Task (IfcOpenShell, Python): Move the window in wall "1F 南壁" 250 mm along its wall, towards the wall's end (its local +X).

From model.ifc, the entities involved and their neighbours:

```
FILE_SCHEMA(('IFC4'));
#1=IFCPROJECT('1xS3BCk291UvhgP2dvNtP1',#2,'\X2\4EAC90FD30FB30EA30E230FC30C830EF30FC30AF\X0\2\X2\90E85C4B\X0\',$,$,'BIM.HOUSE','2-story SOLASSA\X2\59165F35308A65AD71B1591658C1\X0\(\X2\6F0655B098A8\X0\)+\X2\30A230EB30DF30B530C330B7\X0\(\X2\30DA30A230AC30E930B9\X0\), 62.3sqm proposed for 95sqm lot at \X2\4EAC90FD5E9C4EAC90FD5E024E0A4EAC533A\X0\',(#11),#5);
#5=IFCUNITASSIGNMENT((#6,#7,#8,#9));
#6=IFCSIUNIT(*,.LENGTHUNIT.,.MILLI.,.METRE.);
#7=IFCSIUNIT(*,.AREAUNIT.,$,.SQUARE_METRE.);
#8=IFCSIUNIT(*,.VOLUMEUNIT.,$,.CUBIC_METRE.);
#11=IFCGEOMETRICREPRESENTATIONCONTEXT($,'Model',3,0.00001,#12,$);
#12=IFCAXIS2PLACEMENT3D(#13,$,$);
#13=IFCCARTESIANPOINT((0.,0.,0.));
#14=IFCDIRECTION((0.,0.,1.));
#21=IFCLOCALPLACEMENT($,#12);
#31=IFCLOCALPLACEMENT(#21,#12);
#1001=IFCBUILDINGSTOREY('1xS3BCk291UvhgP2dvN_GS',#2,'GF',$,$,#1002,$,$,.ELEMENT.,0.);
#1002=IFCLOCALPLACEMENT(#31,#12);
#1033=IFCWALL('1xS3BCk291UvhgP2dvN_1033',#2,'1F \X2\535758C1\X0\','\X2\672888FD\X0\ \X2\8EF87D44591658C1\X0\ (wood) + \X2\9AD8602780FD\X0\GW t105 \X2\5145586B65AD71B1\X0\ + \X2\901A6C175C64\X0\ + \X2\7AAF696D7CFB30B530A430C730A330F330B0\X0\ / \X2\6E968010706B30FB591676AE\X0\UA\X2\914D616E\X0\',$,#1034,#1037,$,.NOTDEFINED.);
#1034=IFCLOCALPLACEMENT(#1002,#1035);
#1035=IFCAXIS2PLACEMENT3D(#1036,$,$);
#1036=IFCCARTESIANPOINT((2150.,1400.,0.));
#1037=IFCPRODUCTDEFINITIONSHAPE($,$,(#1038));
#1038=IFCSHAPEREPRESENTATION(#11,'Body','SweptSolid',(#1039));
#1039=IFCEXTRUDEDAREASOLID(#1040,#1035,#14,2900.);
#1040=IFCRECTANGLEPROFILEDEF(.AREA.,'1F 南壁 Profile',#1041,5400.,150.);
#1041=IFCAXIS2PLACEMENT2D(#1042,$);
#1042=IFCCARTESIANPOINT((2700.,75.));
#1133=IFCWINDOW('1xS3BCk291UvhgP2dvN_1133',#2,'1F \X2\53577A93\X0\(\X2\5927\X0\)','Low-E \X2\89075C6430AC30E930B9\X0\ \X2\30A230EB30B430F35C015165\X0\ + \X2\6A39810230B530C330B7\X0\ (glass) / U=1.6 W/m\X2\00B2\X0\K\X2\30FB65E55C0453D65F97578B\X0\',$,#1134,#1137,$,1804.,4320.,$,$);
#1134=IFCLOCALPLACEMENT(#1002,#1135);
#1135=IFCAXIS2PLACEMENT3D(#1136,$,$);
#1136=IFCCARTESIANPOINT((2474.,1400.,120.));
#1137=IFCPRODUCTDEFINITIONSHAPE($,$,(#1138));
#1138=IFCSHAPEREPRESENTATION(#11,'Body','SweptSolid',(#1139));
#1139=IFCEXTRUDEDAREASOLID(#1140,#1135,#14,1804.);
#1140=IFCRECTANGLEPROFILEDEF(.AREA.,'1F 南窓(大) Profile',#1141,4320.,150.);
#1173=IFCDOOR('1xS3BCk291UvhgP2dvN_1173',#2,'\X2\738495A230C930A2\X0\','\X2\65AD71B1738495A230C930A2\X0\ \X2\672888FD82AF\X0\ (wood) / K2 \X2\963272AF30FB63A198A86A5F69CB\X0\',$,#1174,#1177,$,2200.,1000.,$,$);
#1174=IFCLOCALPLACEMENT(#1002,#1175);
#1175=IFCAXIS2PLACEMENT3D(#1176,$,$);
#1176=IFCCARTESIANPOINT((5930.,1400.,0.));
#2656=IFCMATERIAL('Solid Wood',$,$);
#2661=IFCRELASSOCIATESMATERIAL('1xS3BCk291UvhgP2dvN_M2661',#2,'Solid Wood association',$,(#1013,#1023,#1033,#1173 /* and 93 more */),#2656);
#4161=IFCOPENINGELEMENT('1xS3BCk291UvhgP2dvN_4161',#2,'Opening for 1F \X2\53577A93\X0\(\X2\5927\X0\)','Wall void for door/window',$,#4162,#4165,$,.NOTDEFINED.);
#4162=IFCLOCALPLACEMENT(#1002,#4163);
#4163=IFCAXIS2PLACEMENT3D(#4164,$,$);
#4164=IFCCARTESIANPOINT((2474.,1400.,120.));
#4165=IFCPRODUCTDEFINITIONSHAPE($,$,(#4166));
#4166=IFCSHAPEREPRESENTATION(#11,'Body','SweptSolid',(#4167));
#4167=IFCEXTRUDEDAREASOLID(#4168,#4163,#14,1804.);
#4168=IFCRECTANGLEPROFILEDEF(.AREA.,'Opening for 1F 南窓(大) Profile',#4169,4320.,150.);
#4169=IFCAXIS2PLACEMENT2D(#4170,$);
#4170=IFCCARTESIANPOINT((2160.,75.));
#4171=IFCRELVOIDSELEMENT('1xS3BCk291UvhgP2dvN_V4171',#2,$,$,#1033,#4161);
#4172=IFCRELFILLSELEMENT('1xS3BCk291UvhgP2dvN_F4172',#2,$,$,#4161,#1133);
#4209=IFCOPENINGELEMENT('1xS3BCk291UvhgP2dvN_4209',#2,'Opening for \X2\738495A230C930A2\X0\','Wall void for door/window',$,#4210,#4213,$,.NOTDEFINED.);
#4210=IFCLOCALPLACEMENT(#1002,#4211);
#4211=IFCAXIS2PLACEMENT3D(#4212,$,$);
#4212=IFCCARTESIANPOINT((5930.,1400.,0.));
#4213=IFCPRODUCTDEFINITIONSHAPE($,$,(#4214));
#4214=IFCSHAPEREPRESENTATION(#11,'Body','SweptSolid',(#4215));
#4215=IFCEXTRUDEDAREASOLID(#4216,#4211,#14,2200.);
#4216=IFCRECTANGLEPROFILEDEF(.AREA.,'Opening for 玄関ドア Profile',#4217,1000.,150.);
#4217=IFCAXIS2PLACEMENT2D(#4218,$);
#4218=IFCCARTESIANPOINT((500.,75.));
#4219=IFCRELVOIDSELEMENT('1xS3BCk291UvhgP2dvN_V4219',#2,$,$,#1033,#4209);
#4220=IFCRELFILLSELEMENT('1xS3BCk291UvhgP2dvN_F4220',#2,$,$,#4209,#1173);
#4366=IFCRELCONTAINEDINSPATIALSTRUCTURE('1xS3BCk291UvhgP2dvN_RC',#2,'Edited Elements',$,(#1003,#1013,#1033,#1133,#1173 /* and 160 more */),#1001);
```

```python
import ifcopenshell
import ifcopenshell.api.geometry
import ifcopenshell.util.placement

model = ifcopenshell.open("model.ifc")

window = model.by_guid("1xS3BCk291UvhgP2dvN_1133")
opening = window.FillsVoids[0].RelatingOpeningElement
wall = opening.VoidsElements[0].RelatingBuildingElement

wall_matrix = ifcopenshell.util.placement.get_local_placement(wall.ObjectPlacement)
shift = wall_matrix[:3, 0] * 250.0
before = ifcopenshell.util.placement.get_local_placement(window.ObjectPlacement)[:3, 3].copy()

# The window is not placed relative to its opening, so move both.
for product in (opening, window):
    matrix = ifcopenshell.util.placement.get_local_placement(product.ObjectPlacement)
    matrix[:3, 3] += shift
    ifcopenshell.api.geometry.edit_object_placement(model, product=product, matrix=matrix, is_si=False)

after = ifcopenshell.util.placement.get_local_placement(window.ObjectPlacement)[:3, 3]
print("window moved by", (after - before).round(3) + 0.0)

model.write("model_rev.ifc")
```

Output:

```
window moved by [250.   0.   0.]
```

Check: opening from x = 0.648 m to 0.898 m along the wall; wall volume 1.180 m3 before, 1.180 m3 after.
